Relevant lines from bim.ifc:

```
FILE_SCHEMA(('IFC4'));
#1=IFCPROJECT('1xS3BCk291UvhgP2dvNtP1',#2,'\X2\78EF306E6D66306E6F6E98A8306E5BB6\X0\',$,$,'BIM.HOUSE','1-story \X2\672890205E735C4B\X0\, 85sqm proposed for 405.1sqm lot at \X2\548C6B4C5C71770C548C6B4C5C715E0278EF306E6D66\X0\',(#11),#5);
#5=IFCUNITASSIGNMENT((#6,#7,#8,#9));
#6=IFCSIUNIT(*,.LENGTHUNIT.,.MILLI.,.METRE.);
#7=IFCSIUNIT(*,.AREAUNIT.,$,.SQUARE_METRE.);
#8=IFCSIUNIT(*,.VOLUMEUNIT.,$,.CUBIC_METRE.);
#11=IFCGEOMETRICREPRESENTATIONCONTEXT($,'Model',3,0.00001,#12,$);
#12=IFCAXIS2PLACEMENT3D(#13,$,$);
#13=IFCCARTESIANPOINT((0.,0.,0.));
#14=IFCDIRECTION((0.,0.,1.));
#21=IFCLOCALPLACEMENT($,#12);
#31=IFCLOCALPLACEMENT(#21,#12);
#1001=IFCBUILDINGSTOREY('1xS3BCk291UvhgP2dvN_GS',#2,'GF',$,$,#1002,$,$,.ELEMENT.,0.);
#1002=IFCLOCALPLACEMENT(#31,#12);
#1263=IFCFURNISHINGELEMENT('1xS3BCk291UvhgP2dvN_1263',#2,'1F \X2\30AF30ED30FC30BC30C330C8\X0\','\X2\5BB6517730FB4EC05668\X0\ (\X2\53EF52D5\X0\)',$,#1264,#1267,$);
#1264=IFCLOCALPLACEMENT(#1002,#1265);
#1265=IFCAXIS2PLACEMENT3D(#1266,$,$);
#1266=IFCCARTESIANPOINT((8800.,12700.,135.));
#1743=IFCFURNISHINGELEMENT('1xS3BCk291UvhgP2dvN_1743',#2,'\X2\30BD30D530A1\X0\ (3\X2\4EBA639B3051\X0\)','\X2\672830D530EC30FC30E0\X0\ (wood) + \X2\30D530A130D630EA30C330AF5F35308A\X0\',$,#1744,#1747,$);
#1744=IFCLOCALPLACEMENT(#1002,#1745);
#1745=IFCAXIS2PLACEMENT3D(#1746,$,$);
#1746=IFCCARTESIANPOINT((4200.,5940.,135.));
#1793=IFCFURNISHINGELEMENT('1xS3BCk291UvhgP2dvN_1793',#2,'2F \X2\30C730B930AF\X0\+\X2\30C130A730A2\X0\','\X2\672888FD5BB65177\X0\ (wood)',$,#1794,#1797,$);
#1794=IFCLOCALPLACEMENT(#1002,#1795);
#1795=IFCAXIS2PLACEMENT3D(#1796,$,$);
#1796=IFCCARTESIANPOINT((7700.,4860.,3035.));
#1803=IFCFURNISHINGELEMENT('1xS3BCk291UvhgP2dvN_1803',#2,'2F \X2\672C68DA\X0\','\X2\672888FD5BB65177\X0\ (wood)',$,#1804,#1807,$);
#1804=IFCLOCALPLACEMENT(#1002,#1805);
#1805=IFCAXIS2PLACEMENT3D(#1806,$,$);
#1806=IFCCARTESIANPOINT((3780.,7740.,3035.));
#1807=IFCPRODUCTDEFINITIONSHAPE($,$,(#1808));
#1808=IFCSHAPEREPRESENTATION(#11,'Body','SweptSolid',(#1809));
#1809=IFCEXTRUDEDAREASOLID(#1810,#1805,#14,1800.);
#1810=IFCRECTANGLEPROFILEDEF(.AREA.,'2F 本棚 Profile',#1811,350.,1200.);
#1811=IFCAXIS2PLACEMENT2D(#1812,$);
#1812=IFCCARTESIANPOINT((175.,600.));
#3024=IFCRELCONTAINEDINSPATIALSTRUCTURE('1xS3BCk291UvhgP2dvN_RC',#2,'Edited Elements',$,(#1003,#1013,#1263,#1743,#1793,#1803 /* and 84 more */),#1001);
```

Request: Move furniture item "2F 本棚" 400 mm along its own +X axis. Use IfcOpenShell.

```python
import ifcopenshell
import ifcopenshell.api.geometry
import ifcopenshell.util.placement
import ifcopenshell.util.unit

model = ifcopenshell.open("bim.ifc")
unit_scale = ifcopenshell.util.unit.calculate_unit_scale(model)

item = model.by_guid("1xS3BCk291UvhgP2dvN_1803")
matrix = ifcopenshell.util.placement.get_local_placement(item.ObjectPlacement)
matrix[:3, 3] += matrix[:3, 0] * 0.4 / unit_scale
ifcopenshell.api.geometry.edit_object_placement(model, product=item, matrix=matrix, is_si=False)

print(ifcopenshell.util.placement.get_local_placement(item.ObjectPlacement).round(3) + 0.0)

model.write("bim_updated.ifc")
```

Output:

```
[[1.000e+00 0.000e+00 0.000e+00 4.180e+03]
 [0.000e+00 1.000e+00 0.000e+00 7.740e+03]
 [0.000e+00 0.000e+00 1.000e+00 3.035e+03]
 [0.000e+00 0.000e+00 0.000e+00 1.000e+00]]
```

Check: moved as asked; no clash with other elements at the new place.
